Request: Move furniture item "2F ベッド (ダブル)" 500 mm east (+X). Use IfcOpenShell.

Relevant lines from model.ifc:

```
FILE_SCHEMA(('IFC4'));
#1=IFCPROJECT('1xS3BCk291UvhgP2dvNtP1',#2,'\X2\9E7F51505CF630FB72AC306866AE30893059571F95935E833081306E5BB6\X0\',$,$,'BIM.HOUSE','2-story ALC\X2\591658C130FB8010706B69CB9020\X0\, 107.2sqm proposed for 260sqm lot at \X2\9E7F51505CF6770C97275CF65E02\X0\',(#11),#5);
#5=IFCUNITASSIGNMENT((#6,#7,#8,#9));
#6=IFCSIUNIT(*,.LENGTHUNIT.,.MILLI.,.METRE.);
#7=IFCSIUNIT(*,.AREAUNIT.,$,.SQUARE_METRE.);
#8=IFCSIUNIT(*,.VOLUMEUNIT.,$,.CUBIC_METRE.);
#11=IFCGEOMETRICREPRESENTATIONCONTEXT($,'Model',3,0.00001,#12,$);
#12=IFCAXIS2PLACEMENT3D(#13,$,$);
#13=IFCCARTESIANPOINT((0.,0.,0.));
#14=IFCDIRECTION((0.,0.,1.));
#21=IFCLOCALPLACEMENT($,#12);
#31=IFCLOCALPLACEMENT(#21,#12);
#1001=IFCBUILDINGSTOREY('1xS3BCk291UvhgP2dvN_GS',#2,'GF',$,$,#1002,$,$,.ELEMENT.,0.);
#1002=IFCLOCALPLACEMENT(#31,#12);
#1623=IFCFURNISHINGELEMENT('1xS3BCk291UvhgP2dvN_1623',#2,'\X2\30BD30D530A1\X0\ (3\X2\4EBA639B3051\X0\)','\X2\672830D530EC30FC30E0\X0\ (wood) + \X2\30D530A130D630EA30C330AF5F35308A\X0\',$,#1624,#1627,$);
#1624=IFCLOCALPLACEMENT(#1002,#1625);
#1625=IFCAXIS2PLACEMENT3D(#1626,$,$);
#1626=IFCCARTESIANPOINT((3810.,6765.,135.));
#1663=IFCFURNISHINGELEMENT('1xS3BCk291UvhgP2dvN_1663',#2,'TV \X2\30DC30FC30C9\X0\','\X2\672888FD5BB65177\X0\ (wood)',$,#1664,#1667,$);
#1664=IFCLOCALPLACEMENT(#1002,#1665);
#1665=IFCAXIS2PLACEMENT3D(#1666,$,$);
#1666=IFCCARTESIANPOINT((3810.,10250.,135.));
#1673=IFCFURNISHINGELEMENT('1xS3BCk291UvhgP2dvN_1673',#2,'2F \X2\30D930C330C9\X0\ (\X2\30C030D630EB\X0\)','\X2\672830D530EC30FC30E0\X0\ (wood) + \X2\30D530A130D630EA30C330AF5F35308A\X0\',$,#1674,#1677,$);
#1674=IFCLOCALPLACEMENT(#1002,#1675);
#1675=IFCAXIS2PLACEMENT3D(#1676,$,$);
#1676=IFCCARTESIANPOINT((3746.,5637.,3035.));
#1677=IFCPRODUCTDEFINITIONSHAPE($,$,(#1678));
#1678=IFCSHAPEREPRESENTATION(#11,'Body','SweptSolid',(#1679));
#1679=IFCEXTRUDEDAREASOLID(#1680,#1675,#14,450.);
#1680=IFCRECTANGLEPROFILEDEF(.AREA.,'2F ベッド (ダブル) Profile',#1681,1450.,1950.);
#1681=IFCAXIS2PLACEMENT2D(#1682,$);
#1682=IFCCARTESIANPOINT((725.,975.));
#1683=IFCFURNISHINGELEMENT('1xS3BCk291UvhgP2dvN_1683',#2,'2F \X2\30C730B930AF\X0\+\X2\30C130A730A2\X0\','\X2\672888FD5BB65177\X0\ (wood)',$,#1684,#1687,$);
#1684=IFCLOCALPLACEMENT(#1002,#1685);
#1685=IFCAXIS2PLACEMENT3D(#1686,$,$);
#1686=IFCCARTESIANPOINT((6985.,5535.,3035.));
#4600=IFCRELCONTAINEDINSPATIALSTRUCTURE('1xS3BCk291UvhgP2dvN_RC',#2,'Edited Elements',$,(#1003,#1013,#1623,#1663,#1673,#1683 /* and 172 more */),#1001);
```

```python
import ifcopenshell
import ifcopenshell.api.geometry
import ifcopenshell.util.placement
import ifcopenshell.util.unit

model = ifcopenshell.open("model.ifc")
unit_scale = ifcopenshell.util.unit.calculate_unit_scale(model)

item = model.by_guid("1xS3BCk291UvhgP2dvN_1673")
matrix = ifcopenshell.util.placement.get_local_placement(item.ObjectPlacement)
matrix[0, 3] += 0.5 / unit_scale
ifcopenshell.api.geometry.edit_object_placement(model, product=item, matrix=matrix, is_si=False)

print(ifcopenshell.util.placement.get_local_placement(item.ObjectPlacement).round(3) + 0.0)

model.write("model_updated.ifc")
```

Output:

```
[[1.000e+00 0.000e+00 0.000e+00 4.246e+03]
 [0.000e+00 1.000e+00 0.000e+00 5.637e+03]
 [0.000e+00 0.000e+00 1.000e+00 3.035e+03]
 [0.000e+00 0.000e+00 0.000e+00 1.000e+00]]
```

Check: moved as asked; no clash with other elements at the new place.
